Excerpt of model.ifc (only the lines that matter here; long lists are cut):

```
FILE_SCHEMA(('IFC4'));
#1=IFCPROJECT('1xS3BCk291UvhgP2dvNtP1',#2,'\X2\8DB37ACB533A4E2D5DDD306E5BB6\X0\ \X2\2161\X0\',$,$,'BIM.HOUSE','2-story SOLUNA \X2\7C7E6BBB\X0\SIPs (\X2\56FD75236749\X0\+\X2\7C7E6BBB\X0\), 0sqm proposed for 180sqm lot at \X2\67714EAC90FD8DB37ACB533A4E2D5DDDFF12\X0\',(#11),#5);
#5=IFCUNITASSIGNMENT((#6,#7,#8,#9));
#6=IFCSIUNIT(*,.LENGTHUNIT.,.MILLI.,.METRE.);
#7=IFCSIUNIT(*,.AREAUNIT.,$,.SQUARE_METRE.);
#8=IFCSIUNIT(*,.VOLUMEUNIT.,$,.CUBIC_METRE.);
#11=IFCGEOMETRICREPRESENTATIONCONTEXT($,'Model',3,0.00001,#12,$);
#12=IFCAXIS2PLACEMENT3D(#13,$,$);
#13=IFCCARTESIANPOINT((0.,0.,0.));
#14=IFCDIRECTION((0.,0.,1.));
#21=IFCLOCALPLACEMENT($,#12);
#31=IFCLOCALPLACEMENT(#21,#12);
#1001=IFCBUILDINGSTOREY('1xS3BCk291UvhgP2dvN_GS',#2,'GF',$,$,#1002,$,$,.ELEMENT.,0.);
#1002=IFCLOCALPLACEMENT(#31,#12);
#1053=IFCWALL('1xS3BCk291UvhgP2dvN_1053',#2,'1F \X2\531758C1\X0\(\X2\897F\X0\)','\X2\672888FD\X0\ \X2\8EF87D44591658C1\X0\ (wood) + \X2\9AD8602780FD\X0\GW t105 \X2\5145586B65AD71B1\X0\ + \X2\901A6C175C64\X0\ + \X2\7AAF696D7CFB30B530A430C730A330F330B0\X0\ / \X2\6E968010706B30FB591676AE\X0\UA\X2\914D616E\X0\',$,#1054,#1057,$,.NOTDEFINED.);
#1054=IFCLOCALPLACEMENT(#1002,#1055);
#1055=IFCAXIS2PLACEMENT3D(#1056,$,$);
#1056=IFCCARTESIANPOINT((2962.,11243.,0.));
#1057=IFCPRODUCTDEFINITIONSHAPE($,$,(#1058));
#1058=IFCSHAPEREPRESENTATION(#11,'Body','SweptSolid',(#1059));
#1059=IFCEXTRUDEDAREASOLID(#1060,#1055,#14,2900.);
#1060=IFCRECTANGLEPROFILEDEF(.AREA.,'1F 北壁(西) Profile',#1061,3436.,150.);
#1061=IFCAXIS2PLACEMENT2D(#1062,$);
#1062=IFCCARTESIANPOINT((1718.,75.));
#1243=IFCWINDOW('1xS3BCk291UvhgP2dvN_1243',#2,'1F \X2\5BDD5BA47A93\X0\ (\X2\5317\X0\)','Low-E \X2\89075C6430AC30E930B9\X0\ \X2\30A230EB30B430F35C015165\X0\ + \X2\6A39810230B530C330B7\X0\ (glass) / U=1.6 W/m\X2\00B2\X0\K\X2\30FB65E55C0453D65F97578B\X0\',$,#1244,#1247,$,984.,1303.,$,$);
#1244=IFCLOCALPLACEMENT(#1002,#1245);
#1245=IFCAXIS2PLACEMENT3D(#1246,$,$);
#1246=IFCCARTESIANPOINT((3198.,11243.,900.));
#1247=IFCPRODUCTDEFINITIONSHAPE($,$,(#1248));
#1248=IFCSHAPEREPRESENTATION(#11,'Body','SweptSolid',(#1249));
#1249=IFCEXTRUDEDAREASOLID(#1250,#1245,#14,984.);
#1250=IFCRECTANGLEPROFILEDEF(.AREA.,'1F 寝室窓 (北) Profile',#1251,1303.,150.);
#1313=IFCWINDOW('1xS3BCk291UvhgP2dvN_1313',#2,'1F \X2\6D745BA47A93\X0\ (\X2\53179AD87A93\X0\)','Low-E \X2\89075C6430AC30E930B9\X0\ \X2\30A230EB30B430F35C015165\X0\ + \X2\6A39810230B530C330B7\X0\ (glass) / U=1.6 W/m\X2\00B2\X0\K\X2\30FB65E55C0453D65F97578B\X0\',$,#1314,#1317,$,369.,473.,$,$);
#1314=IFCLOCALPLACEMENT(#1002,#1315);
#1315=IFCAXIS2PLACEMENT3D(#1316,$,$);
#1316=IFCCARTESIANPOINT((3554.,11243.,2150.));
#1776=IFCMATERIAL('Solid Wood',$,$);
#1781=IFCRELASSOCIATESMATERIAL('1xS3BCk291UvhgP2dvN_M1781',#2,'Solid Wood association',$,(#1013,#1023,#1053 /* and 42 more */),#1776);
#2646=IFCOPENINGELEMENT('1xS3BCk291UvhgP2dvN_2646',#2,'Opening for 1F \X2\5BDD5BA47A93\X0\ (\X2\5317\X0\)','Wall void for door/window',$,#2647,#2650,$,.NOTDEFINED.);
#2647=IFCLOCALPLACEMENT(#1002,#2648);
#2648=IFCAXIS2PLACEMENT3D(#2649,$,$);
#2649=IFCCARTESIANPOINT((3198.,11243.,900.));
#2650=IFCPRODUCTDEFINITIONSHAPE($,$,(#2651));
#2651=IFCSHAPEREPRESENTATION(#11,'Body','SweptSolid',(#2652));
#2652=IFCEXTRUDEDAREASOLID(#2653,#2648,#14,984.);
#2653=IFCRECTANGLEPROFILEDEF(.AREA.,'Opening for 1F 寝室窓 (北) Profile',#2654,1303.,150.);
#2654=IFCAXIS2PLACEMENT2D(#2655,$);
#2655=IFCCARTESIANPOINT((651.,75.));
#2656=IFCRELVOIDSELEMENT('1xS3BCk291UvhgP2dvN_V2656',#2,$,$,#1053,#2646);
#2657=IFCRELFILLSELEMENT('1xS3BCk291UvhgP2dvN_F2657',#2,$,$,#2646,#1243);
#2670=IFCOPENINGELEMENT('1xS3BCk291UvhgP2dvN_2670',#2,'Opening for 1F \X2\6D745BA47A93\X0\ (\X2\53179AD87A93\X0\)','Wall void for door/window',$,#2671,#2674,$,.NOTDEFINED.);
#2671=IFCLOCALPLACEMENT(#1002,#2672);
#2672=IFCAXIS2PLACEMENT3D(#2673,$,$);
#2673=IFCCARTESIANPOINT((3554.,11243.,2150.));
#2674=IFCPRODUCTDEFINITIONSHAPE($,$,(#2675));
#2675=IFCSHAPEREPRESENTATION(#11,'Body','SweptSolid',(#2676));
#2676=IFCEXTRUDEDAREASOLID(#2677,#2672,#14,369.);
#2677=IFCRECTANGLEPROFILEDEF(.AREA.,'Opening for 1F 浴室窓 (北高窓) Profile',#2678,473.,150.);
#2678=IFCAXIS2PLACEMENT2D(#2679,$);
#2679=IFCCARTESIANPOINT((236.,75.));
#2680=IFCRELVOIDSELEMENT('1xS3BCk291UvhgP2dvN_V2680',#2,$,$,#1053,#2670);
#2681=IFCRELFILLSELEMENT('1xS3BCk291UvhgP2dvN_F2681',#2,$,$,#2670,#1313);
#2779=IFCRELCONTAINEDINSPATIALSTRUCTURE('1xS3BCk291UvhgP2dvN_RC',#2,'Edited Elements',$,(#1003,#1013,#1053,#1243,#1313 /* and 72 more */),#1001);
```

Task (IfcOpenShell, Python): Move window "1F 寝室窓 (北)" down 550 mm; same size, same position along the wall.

```python
import numpy as np
import ifcopenshell
import ifcopenshell.api.geometry
import ifcopenshell.util.placement
import ifcopenshell.util.unit

model = ifcopenshell.open("model.ifc")
unit_scale = ifcopenshell.util.unit.calculate_unit_scale(model)

window = model.by_id(1243)
opening = window.FillsVoids[0].RelatingOpeningElement
dz = -0.55 / unit_scale

shift = np.array([0.0, 0.0, dz])
# The window is not placed relative to its opening, so move both.
for product in (opening, window):
    matrix = ifcopenshell.util.placement.get_local_placement(product.ObjectPlacement)
    matrix[:3, 3] += shift
    ifcopenshell.api.geometry.edit_object_placement(model, product=product, matrix=matrix, is_si=False)

print(f"moved by {dz * unit_scale:+.3f} m")

model.write("model-out.ifc")
```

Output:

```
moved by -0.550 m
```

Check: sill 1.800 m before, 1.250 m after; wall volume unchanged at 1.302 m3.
